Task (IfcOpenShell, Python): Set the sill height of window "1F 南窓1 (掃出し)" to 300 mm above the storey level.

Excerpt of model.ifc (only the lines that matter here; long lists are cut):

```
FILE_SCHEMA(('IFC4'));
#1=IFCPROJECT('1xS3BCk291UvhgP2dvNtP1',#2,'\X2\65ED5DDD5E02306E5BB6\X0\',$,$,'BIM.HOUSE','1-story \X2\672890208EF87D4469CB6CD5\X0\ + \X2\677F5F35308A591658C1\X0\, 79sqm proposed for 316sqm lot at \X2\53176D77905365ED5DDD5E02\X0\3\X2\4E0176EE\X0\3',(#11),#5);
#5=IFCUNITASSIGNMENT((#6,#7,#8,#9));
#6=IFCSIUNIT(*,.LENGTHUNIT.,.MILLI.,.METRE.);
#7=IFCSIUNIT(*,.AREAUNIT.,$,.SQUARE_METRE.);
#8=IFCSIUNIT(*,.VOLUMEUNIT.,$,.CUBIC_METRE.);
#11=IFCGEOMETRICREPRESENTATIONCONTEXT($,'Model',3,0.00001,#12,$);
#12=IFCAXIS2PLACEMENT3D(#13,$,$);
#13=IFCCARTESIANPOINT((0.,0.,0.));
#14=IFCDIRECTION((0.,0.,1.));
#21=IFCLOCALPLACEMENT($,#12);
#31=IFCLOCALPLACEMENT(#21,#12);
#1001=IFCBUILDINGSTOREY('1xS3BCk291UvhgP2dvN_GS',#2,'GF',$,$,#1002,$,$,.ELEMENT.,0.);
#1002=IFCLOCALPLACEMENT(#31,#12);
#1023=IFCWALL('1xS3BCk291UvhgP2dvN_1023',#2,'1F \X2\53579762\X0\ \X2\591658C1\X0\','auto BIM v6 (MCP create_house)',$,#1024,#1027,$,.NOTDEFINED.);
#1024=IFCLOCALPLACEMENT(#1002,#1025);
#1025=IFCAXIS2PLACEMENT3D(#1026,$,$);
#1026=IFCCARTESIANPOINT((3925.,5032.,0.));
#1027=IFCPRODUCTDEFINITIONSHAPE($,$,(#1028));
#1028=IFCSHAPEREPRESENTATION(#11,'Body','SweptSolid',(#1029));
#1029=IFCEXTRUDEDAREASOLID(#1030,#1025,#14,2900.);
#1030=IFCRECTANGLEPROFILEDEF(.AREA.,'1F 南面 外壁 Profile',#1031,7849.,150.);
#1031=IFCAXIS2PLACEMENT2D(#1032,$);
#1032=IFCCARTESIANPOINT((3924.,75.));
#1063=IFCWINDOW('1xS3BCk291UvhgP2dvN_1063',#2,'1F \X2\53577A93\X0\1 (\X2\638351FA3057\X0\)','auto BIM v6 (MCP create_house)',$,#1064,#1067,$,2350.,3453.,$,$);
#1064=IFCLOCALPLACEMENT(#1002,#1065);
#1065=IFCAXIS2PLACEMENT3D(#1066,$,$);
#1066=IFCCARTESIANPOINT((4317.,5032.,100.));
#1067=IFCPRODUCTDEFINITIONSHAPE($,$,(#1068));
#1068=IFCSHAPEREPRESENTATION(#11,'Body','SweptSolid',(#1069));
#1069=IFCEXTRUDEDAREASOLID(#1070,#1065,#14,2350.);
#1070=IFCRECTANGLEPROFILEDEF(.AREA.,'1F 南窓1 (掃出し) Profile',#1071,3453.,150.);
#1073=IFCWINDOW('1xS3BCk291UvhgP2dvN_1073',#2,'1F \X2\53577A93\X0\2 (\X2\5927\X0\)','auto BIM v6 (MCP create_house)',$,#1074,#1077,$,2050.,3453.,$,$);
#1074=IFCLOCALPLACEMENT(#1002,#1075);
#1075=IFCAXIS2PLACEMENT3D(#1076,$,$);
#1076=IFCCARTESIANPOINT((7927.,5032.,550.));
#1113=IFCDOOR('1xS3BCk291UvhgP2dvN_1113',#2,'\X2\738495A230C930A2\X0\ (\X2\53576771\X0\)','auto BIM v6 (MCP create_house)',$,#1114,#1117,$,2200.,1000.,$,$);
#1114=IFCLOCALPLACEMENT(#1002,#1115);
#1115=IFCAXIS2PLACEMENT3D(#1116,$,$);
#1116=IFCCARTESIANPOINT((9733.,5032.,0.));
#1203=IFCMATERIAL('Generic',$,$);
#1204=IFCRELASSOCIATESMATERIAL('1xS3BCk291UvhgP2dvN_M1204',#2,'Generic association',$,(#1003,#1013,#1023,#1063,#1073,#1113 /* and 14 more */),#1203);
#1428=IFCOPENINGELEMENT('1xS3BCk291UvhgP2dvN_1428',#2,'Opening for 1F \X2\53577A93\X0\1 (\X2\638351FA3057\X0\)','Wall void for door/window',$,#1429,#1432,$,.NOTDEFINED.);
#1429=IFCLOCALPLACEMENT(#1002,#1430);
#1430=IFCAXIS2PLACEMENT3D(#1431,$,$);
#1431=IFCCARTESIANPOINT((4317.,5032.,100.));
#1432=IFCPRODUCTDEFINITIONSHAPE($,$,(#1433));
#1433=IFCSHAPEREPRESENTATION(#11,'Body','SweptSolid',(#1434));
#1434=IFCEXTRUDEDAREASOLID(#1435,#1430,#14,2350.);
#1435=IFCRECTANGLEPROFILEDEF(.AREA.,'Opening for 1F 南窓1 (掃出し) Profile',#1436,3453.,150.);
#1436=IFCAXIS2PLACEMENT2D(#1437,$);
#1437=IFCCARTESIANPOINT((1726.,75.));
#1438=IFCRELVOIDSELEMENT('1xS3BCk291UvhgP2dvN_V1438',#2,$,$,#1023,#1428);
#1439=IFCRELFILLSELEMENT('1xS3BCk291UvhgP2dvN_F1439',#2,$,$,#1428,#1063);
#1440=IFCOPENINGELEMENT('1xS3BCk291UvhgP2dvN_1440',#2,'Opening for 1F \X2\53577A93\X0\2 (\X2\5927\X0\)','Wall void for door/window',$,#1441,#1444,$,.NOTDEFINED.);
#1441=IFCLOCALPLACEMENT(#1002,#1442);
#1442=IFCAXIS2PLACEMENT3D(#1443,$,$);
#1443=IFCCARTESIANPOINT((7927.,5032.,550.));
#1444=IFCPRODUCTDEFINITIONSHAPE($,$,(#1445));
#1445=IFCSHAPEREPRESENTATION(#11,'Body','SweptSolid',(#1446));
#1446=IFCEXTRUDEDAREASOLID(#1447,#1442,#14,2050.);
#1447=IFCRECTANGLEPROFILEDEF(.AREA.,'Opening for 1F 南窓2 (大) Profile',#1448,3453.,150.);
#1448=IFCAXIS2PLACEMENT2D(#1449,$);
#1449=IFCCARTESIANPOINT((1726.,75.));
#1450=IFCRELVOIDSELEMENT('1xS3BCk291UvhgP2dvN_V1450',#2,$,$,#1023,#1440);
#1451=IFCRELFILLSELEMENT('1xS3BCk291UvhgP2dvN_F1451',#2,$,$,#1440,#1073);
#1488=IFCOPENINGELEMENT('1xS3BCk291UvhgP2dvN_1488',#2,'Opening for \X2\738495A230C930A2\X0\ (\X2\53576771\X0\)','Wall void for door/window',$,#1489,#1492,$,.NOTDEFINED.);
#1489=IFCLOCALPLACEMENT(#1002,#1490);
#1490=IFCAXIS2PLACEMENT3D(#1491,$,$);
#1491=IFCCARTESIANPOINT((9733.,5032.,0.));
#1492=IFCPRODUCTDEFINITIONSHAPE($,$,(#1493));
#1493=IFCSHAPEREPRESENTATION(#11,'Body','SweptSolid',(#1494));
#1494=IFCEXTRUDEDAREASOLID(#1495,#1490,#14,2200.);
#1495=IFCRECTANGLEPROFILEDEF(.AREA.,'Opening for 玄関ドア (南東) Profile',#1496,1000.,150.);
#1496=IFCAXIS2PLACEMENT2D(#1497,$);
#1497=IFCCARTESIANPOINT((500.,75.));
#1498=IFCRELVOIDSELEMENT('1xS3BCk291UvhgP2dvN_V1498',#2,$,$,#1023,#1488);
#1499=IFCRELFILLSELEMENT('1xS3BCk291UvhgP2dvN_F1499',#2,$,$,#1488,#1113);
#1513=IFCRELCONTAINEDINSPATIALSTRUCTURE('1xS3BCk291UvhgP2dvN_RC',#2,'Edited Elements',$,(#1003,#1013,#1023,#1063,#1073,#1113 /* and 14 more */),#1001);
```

```python
import numpy as np
import ifcopenshell
import ifcopenshell.api.geometry
import ifcopenshell.geom
import ifcopenshell.util.element
import ifcopenshell.util.placement
import ifcopenshell.util.shape
import ifcopenshell.util.unit

model = ifcopenshell.open("model.ifc")
unit_scale = ifcopenshell.util.unit.calculate_unit_scale(model)

window = model.by_guid("1xS3BCk291UvhgP2dvN_1063")
opening = window.FillsVoids[0].RelatingOpeningElement
storey = ifcopenshell.util.element.get_container(window, ifc_class="IfcBuildingStorey")
level = ifcopenshell.util.placement.get_local_placement(storey.ObjectPlacement)[2, 3]

# The opening's origin need not be at the sill, so measure its lowest point.
shape = ifcopenshell.geom.create_shape(ifcopenshell.geom.settings(), opening)
bottom = ifcopenshell.util.shape.get_shape_bottom_elevation(shape, shape.geometry) / unit_scale
dz = level + 0.3 / unit_scale - bottom

shift = np.array([0.0, 0.0, dz])
# The window is not placed relative to its opening, so move both.
for product in (opening, window):
    matrix = ifcopenshell.util.placement.get_local_placement(product.ObjectPlacement)
    matrix[:3, 3] += shift
    ifcopenshell.api.geometry.edit_object_placement(model, product=product, matrix=matrix, is_si=False)

print(f"moved by {dz * unit_scale:+.3f} m")

model.write("model_rev.ifc")
```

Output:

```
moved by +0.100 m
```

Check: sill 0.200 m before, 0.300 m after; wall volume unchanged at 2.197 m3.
